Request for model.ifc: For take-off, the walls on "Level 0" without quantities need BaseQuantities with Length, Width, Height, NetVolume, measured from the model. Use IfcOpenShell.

First a look at what the model holds.

```python
import ifcopenshell
import ifcopenshell.util.element
import ifcopenshell.util.unit

model = ifcopenshell.open("model.ifc")
print(model.schema)
for unit_type in ("LENGTHUNIT", "AREAUNIT", "VOLUMEUNIT"):
    print(unit_type, ifcopenshell.util.unit.calculate_unit_scale(model, unit_type))
storey = next(s for s in model.by_type("IfcBuildingStorey") if s.Name == "Level 0")
walls = [e for e in ifcopenshell.util.element.get_decomposition(storey) if e.is_a("IfcWall")]
for e in sorted(walls, key=lambda e: e.id()):
    print(e.id(), e.is_a(), e.Name, list(ifcopenshell.util.element.get_psets(e, qtos_only=True)), sep=" | ")
```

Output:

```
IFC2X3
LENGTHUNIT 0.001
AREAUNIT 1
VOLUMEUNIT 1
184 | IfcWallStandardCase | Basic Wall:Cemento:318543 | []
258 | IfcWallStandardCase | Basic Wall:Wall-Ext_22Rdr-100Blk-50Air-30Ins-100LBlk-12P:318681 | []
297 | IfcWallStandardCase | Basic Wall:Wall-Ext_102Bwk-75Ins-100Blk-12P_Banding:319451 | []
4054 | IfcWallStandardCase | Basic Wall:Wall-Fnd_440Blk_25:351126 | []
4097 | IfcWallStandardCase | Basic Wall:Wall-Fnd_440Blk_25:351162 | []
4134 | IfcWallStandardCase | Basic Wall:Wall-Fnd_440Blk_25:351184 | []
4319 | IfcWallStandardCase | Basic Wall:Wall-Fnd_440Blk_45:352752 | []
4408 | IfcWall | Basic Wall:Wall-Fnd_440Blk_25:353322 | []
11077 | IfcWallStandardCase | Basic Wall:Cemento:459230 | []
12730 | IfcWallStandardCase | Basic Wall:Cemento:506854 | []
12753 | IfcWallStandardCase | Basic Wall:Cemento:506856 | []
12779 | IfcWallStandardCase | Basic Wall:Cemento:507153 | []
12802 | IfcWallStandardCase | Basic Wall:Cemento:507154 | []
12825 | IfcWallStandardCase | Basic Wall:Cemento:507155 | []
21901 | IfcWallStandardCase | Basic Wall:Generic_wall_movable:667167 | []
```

```python
import ifcopenshell
import ifcopenshell.api.pset
import ifcopenshell.geom
import ifcopenshell.util.element
import ifcopenshell.util.shape
import ifcopenshell.util.unit

model = ifcopenshell.open("model.ifc")
unit_scale = ifcopenshell.util.unit.calculate_unit_scale(model)
volume_scale = ifcopenshell.util.unit.calculate_unit_scale(model, "VOLUMEUNIT")
settings = ifcopenshell.geom.settings()

storey = next(s for s in model.by_type("IfcBuildingStorey") if s.Name == "Level 0")
walls = [e for e in ifcopenshell.util.element.get_decomposition(storey) if e.is_a("IfcWall")]

for e in sorted(walls, key=lambda e: e.id()):
    if ifcopenshell.util.element.get_psets(e, qtos_only=True, should_inherit=False):
        continue
    # Geometry comes back in metres, in the element's own axes.
    shape = ifcopenshell.geom.create_shape(settings, e)
    values = {
        "Length": ifcopenshell.util.shape.get_x(shape.geometry) / unit_scale,
        "Width": ifcopenshell.util.shape.get_y(shape.geometry) / unit_scale,
        "Height": ifcopenshell.util.shape.get_z(shape.geometry) / unit_scale,
        "NetVolume": ifcopenshell.util.shape.get_volume(shape.geometry) / volume_scale,
    }
    qto = ifcopenshell.api.pset.add_qto(model, product=e, name="BaseQuantities")
    ifcopenshell.api.pset.edit_qto(model, qto=qto, properties=values)
    print(e.id(), {k: round(v, 3) for k, v in values.items()})

model.write("model_rev.ifc")
```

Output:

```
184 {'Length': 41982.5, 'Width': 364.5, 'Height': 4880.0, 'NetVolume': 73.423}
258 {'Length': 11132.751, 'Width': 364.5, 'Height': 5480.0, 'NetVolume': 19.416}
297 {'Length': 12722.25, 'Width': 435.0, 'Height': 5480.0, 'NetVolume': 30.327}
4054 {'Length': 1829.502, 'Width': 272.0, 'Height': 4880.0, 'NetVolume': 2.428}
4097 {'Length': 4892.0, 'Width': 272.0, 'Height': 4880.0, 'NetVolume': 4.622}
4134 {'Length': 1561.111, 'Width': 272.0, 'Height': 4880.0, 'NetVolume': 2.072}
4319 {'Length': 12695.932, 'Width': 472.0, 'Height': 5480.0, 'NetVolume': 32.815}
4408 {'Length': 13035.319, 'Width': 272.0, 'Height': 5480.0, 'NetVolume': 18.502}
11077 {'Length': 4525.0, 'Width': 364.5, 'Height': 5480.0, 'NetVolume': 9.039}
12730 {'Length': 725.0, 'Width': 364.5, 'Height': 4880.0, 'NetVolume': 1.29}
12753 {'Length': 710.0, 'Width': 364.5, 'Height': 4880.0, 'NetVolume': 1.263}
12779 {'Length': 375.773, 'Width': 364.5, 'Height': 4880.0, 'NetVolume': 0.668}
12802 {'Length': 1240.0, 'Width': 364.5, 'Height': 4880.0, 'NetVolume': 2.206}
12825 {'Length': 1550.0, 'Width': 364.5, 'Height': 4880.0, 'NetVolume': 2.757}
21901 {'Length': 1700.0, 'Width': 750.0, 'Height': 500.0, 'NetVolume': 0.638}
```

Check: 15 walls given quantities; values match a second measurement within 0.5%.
